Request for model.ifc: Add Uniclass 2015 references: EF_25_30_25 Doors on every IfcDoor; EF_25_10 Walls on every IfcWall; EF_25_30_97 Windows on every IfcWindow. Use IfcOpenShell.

First a look at what the model holds.

```python
import ifcopenshell

model = ifcopenshell.open("model.ifc")
print(model.schema)
print("classifications:", [c.Name for c in model.by_type("IfcClassification")])
for ifc_class in ("IfcDoor", "IfcRoof", "IfcStair", "IfcWall", "IfcWindow"):
    print(ifc_class, len(model.by_type(ifc_class)))
```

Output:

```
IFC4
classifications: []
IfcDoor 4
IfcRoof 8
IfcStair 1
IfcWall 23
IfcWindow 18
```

```python
import ifcopenshell
import ifcopenshell.api.classification

model = ifcopenshell.open("model.ifc")

system = ifcopenshell.api.classification.add_classification(model, classification="Uniclass 2015")

codes = {
    "IfcDoor": ("EF_25_30_25", "Doors"),
    "IfcWall": ("EF_25_10", "Walls"),
    "IfcWindow": ("EF_25_30_97", "Windows"),
}
for ifc_class, (code, name) in codes.items():
    products = model.by_type(ifc_class)
    ifcopenshell.api.classification.add_reference(
        model, products=products, classification=system, identification=code, name=name
    )
    print(code, len(products))

model.write("model_edited.ifc")
```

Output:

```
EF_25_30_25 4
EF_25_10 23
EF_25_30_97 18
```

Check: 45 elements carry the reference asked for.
